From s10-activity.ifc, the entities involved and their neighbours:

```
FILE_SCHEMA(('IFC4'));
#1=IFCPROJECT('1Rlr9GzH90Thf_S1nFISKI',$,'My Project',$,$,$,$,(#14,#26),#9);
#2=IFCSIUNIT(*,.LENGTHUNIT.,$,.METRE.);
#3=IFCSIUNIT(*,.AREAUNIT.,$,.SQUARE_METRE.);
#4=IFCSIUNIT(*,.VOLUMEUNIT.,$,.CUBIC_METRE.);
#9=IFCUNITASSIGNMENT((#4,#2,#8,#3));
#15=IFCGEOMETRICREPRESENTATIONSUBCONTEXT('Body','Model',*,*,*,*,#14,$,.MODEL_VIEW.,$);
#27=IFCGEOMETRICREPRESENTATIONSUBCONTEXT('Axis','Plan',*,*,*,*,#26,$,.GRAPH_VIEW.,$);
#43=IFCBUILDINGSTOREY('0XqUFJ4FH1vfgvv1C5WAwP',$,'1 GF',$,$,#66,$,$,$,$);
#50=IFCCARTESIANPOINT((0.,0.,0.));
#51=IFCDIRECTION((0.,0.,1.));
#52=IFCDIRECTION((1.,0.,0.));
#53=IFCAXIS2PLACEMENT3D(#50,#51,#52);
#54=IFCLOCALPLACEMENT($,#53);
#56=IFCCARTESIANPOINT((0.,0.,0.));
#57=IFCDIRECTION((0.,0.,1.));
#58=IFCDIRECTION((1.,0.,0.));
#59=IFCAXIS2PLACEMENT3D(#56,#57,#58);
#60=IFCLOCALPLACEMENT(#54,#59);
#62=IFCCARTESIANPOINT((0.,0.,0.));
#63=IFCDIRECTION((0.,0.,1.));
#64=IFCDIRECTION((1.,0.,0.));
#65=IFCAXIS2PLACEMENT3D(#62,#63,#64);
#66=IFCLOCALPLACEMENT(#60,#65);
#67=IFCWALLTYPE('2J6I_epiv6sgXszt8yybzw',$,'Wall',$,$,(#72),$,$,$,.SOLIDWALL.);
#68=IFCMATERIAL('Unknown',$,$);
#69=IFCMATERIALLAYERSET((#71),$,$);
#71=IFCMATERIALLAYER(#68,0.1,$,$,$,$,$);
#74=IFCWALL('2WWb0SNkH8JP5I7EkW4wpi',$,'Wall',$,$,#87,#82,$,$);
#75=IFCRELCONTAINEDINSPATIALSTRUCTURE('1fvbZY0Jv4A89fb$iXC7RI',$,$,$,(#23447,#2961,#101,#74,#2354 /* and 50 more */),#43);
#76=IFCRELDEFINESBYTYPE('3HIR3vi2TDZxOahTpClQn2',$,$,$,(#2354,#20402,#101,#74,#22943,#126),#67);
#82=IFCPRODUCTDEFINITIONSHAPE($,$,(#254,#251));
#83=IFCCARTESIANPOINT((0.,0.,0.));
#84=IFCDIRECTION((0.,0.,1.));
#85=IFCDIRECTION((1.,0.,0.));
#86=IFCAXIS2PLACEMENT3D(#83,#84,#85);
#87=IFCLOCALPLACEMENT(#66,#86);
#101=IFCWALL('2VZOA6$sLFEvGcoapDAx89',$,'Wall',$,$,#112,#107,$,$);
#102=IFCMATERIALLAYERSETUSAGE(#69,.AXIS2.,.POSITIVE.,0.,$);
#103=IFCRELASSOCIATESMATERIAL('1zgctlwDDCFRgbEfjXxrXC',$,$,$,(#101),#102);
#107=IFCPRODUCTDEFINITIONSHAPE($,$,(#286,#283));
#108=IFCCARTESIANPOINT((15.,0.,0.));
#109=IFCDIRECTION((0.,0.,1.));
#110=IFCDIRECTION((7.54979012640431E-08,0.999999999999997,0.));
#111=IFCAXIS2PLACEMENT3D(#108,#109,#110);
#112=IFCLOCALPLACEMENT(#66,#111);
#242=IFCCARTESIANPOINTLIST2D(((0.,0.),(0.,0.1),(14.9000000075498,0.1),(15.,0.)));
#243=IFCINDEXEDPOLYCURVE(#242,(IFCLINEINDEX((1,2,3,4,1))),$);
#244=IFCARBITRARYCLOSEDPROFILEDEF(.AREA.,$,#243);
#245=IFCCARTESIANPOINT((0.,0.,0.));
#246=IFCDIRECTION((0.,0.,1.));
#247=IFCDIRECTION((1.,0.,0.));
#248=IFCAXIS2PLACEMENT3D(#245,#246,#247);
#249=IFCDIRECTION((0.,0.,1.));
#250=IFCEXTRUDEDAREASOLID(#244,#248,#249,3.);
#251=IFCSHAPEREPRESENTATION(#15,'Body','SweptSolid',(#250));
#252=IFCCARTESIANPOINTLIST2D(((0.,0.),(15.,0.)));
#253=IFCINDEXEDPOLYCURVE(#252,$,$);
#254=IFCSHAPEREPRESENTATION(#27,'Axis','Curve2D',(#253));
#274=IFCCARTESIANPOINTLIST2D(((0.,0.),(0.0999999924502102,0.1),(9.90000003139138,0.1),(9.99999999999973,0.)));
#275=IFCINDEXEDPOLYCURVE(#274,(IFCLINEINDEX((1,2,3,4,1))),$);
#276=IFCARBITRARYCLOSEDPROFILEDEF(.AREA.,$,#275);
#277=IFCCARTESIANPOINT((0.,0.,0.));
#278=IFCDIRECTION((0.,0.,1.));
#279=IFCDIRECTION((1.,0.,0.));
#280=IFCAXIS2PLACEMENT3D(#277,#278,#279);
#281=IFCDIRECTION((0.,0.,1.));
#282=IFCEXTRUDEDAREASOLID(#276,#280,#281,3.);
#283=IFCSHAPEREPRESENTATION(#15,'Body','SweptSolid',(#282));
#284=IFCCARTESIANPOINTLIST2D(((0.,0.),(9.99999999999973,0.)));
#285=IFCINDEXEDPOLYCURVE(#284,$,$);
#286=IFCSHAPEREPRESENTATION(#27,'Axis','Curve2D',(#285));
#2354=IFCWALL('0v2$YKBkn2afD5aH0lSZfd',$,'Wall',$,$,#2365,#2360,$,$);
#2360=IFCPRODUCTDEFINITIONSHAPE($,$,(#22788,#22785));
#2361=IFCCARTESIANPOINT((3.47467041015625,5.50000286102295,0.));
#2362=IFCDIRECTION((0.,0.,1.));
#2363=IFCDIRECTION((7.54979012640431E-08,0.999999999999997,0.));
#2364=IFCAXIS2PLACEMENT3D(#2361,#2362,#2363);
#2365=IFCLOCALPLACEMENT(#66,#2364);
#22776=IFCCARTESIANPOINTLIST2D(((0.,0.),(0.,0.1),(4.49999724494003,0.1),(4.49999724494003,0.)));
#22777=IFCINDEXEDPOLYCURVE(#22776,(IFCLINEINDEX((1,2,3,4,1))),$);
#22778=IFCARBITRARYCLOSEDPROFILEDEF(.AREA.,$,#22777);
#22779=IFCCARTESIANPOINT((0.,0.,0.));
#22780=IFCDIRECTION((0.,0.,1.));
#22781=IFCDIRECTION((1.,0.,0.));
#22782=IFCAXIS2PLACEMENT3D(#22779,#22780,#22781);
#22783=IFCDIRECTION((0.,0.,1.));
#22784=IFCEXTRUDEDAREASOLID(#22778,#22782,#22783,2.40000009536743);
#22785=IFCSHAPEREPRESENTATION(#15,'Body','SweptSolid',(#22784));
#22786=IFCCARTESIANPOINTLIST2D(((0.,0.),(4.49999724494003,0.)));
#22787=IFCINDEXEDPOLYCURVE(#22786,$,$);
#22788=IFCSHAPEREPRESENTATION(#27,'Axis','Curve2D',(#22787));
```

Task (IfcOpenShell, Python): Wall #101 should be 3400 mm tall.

```python
import ifcopenshell
import ifcopenshell.geom
import ifcopenshell.util.representation
import ifcopenshell.util.shape
import ifcopenshell.util.unit

model = ifcopenshell.open("s10-activity.ifc")
unit_scale = ifcopenshell.util.unit.calculate_unit_scale(model)
settings = ifcopenshell.geom.settings()


def volume(element):
    """Net volume in cubic metres, openings subtracted."""
    shape = ifcopenshell.geom.create_shape(settings, element)
    return ifcopenshell.util.shape.get_volume(shape.geometry)


wall = model.by_guid("2VZOA6$sLFEvGcoapDAx89")
before = volume(wall)

body = ifcopenshell.util.representation.get_representation(wall, "Model", "Body")
solid = body.Items[0]
old_height = solid.Depth
solid.Depth = 3.4 / unit_scale
after = volume(wall)

print(f"height {old_height:g} -> {solid.Depth:g}, volume {before:.3f} -> {after:.3f} m3")

model.write("s10-activity_edited.ifc")
```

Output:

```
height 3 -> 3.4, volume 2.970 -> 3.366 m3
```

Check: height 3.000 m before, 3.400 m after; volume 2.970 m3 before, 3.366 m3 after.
